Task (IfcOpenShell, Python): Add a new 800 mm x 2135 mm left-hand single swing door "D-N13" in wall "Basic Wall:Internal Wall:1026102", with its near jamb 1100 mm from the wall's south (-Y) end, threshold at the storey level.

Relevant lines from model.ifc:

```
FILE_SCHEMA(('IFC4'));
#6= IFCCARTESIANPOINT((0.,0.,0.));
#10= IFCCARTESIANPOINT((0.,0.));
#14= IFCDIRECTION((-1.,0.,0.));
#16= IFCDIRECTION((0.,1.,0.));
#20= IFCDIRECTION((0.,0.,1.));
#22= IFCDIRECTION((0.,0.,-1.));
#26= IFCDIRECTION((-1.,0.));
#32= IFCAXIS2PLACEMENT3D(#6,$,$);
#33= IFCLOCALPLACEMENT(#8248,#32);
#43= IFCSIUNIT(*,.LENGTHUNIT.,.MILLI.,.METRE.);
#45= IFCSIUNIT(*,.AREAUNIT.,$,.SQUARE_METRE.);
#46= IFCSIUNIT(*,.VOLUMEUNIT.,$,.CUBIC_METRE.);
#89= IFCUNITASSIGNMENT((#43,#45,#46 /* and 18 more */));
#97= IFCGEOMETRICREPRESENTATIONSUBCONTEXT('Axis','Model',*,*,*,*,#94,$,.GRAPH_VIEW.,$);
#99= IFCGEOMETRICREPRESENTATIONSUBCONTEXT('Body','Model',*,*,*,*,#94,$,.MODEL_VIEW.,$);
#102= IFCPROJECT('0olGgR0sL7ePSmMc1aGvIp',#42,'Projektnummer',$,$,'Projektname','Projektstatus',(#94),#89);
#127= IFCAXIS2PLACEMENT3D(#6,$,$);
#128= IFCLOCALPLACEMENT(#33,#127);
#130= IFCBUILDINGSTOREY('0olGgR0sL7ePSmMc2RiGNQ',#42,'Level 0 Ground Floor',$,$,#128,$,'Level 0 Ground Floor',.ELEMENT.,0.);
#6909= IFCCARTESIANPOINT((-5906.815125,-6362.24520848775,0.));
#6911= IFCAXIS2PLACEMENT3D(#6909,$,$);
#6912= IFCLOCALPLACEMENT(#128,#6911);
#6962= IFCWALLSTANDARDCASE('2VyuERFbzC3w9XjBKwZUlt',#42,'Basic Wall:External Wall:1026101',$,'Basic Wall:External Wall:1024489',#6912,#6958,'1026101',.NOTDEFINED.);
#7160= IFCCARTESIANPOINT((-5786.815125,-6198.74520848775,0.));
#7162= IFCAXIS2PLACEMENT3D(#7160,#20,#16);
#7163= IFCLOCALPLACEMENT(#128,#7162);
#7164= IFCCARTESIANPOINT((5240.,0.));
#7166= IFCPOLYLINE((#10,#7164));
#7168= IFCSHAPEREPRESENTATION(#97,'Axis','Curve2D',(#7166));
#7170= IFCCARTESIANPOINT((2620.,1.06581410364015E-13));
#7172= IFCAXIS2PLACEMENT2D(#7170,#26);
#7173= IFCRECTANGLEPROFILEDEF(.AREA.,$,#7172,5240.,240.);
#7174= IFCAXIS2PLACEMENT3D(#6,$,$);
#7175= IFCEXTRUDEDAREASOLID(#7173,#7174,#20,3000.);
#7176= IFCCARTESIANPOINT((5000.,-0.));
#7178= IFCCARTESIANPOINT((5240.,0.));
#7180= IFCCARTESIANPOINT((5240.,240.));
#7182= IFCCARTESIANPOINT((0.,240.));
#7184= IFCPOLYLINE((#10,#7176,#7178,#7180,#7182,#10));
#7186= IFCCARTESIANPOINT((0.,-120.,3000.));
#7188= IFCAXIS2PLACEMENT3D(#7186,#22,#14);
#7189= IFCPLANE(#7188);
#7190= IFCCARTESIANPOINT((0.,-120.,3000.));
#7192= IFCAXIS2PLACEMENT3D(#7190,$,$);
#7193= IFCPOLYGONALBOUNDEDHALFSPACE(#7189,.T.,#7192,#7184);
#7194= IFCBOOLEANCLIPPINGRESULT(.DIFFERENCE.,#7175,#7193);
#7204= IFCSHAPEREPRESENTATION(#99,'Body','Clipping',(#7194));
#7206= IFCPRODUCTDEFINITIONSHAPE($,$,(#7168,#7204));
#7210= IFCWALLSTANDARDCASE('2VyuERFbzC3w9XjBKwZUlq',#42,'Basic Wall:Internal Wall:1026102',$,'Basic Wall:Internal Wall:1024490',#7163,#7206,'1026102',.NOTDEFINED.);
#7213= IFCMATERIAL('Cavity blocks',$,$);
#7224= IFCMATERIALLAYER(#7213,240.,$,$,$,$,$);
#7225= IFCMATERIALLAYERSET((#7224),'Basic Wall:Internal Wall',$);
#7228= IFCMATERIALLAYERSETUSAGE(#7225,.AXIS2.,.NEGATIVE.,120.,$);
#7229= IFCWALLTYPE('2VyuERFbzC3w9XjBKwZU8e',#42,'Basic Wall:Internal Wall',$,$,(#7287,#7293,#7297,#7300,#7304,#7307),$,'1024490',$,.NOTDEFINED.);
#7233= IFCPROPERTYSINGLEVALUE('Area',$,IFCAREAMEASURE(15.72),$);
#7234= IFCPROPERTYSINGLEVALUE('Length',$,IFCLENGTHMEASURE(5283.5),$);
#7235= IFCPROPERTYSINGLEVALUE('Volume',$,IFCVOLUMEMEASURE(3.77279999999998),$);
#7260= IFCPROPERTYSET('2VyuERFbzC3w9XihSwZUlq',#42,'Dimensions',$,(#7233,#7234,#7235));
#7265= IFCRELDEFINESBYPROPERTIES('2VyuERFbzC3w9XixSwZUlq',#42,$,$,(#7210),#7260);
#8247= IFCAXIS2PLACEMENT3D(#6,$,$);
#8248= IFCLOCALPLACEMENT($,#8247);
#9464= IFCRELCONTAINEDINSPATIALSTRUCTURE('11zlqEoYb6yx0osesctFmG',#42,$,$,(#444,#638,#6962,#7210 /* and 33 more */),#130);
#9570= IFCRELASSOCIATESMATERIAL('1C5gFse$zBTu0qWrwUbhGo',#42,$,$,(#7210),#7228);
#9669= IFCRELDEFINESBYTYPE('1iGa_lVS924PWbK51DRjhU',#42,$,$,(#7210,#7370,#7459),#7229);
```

```python
import numpy as np
import ifcopenshell
import ifcopenshell.api.feature
import ifcopenshell.api.geometry
import ifcopenshell.api.pset
import ifcopenshell.api.root
import ifcopenshell.api.spatial
import ifcopenshell.geom
import ifcopenshell.util.element
import ifcopenshell.util.placement
import ifcopenshell.util.representation
import ifcopenshell.util.shape
import ifcopenshell.util.unit

model = ifcopenshell.open("model.ifc")
unit_scale = ifcopenshell.util.unit.calculate_unit_scale(model)
area_scale = ifcopenshell.util.unit.calculate_unit_scale(model, "AREAUNIT")
volume_scale = ifcopenshell.util.unit.calculate_unit_scale(model, "VOLUMEUNIT")
settings = ifcopenshell.geom.settings()


def volume(element):
    """Net volume in cubic metres, openings subtracted."""
    shape = ifcopenshell.geom.create_shape(settings, element)
    return ifcopenshell.util.shape.get_volume(shape.geometry)


wall = model.by_guid("2VyuERFbzC3w9XjBKwZUlq")
storey = ifcopenshell.util.element.get_container(wall, ifc_class="IfcBuildingStorey")
context = ifcopenshell.util.representation.get_context(model, "Model", "Body", "MODEL_VIEW")
before = volume(wall)

width, height, from_end, sill = 0.8, 2.135, 1.1, 0.0  # metres

# The wall runs along its own X axis, and the end named is its -X end.
wall_shape = ifcopenshell.geom.create_shape(settings, wall)
x, y, z = ifcopenshell.util.shape.get_vertices(wall_shape.geometry).T
start = x.min() + from_end
face, thickness = float(y.min()), float(y.max() - y.min())
wall_matrix = ifcopenshell.util.placement.get_local_placement(wall.ObjectPlacement)
level = ifcopenshell.util.placement.get_local_placement(storey.ObjectPlacement)[2, 3]


def in_wall(x, y):
    """Placement at x, y metres in the wall's axes, at sill height."""
    matrix = wall_matrix.copy()
    matrix[:, 3] = wall_matrix @ np.array([x / unit_scale, y / unit_scale, 0.0, 1.0])
    matrix[2, 3] = level + sill / unit_scale
    return matrix


# Opening: a box that overshoots both wall faces by 50 mm.
opening = ifcopenshell.api.root.create_entity(model, ifc_class="IfcOpeningElement", predefined_type="OPENING")
box = ifcopenshell.api.geometry.add_wall_representation(
    model, context=context, length=width, height=height, thickness=thickness + 0.1
)
ifcopenshell.api.geometry.assign_representation(model, product=opening, representation=box)
ifcopenshell.api.geometry.edit_object_placement(model, product=opening, matrix=in_wall(start, face - 0.05), is_si=False)
ifcopenshell.api.feature.add_feature(model, feature=opening, element=wall)

door = ifcopenshell.api.root.create_entity(model, ifc_class="IfcDoor", name="D-N13", predefined_type="DOOR")
door.OverallWidth, door.OverallHeight = width / unit_scale, height / unit_scale
door.OperationType = "SINGLE_SWING_LEFT"
body = ifcopenshell.api.geometry.add_door_representation(
    model,
    context=context,
    overall_width=door.OverallWidth,
    overall_height=door.OverallHeight,
    operation_type="SINGLE_SWING_LEFT",
    lining_properties={"LiningDepth": thickness / unit_scale, "ThresholdDepth": thickness / unit_scale},
)
ifcopenshell.api.geometry.assign_representation(model, product=door, representation=body)
ifcopenshell.api.spatial.assign_container(model, products=[door], relating_structure=storey)
ifcopenshell.api.feature.add_filling(model, opening=opening, element=door)

# The lining spans the wall, so the door starts at the wall face.
ifcopenshell.api.geometry.edit_object_placement(model, product=door, matrix=in_wall(start, face), is_si=False)

after = volume(wall)

# Update the wall's stored quantities.
pset = model.by_id(ifcopenshell.util.element.get_pset(wall, "Dimensions", should_inherit=False)["id"])
ifcopenshell.api.pset.edit_pset(model, pset=pset, properties={
    "Area": model.create_entity("IfcAreaMeasure", after / thickness / area_scale),
    "Volume": model.create_entity("IfcVolumeMeasure", after / volume_scale),
})

print(f"wall volume {before:.3f} -> {after:.3f} m3")

model.write("model_rev.ifc")
```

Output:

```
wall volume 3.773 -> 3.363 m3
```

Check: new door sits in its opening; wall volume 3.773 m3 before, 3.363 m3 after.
